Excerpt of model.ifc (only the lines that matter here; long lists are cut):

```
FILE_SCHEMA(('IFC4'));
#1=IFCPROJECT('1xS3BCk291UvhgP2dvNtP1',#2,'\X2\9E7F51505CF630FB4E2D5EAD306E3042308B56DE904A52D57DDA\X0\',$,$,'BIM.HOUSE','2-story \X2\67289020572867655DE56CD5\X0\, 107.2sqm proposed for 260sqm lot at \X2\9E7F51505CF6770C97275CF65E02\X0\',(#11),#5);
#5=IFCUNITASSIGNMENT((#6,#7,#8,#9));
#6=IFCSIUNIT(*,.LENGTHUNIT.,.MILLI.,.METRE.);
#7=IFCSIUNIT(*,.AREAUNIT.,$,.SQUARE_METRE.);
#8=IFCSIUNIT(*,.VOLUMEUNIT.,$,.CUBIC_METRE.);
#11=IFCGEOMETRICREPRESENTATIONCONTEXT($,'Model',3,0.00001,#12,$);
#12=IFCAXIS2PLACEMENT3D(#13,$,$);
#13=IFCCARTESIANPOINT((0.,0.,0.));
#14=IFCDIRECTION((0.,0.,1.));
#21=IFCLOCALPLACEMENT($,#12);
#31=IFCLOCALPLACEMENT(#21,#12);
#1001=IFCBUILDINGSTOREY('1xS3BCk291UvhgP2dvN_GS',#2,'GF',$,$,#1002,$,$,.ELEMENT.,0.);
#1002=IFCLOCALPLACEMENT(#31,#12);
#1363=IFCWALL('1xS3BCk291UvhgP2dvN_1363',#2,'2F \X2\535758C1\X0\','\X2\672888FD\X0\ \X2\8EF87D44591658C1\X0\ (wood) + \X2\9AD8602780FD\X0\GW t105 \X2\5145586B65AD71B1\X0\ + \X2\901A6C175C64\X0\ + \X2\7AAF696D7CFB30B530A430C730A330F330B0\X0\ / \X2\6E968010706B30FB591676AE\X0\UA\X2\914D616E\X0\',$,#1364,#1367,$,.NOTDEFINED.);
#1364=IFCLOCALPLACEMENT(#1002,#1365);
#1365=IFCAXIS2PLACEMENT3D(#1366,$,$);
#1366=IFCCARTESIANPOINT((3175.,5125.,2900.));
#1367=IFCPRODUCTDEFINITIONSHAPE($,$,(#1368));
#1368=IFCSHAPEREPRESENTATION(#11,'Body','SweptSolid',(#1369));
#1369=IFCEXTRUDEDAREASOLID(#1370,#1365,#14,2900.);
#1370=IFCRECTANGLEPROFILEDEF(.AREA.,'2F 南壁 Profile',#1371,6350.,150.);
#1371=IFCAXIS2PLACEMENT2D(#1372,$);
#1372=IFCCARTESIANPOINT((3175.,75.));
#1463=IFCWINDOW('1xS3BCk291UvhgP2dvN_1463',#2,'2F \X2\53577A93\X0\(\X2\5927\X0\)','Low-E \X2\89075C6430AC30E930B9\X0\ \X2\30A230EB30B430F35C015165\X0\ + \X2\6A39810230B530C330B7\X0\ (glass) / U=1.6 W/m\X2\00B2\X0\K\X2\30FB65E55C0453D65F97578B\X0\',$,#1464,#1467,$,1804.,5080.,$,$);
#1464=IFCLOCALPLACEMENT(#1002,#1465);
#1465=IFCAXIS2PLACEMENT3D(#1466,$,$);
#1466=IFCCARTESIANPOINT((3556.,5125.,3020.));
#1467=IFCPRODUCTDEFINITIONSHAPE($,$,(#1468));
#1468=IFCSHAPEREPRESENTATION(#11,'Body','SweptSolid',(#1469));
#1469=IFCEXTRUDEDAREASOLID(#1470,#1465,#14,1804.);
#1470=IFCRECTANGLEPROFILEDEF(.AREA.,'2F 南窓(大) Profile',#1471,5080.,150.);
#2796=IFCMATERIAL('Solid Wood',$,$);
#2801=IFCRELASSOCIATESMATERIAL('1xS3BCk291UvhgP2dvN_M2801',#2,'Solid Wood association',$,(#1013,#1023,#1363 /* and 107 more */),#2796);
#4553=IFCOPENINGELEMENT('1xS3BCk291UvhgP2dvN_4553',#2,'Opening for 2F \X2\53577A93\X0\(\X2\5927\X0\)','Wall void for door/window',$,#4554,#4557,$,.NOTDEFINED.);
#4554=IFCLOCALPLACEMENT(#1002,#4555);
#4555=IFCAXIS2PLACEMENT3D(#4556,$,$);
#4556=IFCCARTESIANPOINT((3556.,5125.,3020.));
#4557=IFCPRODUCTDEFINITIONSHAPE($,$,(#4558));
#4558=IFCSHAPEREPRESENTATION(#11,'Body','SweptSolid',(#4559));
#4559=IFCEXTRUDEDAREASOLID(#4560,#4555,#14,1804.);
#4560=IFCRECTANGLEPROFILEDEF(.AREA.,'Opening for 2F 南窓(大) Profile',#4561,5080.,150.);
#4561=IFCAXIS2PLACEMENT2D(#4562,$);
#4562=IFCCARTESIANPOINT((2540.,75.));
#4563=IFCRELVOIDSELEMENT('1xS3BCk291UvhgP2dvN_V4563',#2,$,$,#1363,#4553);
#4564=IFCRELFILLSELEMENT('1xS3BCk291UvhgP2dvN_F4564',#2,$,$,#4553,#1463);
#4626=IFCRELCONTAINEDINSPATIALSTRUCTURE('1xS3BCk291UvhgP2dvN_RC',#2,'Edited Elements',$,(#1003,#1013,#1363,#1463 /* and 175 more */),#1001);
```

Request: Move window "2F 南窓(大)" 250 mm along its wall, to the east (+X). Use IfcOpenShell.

```python
import ifcopenshell
import ifcopenshell.api.geometry
import ifcopenshell.util.placement
import ifcopenshell.util.unit

model = ifcopenshell.open("model.ifc")
unit_scale = ifcopenshell.util.unit.calculate_unit_scale(model)

window = model.by_guid("1xS3BCk291UvhgP2dvN_1463")
opening = window.FillsVoids[0].RelatingOpeningElement
wall = opening.VoidsElements[0].RelatingBuildingElement

wall_matrix = ifcopenshell.util.placement.get_local_placement(wall.ObjectPlacement)
shift = wall_matrix[:3, 0] * 0.25 / unit_scale
before = ifcopenshell.util.placement.get_local_placement(window.ObjectPlacement)[:3, 3].copy()

# The window is not placed relative to its opening, so move both.
for product in (opening, window):
    matrix = ifcopenshell.util.placement.get_local_placement(product.ObjectPlacement)
    matrix[:3, 3] += shift
    ifcopenshell.api.geometry.edit_object_placement(model, product=product, matrix=matrix, is_si=False)

after = ifcopenshell.util.placement.get_local_placement(window.ObjectPlacement)[:3, 3]
print("window moved by", (after - before).round(3) + 0.0)

model.write("model_edited.ifc")
```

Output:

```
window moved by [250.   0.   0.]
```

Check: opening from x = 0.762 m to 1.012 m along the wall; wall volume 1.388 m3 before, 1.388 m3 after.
